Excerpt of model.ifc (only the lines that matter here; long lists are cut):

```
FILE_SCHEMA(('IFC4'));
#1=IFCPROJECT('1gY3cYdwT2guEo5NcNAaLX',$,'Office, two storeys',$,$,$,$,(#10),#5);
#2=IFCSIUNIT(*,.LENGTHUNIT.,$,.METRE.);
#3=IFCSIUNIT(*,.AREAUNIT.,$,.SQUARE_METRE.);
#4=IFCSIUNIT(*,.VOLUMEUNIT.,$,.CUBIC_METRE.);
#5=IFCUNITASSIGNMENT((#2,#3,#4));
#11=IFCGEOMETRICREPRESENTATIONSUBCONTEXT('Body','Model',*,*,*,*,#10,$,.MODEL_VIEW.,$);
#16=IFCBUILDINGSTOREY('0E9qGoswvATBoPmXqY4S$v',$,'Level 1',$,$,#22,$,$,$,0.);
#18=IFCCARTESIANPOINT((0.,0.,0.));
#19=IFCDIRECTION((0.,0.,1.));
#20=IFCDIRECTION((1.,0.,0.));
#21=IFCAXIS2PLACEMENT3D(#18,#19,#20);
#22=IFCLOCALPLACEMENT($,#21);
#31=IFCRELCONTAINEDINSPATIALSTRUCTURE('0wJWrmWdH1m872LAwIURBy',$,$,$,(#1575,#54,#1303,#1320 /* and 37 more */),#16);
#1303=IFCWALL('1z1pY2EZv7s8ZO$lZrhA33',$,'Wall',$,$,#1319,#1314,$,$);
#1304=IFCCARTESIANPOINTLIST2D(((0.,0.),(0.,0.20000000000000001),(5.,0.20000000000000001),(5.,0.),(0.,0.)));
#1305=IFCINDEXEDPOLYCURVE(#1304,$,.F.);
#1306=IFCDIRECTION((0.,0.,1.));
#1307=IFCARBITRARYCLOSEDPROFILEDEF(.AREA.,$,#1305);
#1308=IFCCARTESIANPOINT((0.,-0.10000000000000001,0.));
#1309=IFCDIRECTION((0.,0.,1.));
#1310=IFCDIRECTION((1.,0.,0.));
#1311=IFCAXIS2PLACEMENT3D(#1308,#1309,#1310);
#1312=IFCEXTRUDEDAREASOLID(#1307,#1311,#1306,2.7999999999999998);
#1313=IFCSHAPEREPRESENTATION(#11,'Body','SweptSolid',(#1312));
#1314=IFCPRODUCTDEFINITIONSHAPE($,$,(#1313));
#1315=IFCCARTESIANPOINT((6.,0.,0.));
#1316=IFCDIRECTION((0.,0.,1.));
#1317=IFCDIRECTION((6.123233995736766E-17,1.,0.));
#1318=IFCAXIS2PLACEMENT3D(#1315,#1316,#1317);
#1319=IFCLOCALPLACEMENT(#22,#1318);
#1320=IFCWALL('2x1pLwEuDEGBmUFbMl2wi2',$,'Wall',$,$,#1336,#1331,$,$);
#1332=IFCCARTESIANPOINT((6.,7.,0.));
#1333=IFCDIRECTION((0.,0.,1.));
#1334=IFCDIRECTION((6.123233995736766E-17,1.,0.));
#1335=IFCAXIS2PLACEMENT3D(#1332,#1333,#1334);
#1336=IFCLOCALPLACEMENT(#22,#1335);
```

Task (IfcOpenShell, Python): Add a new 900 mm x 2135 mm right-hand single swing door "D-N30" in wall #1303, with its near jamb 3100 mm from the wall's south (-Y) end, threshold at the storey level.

```python
import numpy as np
import ifcopenshell
import ifcopenshell.api.feature
import ifcopenshell.api.geometry
import ifcopenshell.api.root
import ifcopenshell.api.spatial
import ifcopenshell.geom
import ifcopenshell.util.element
import ifcopenshell.util.placement
import ifcopenshell.util.representation
import ifcopenshell.util.shape
import ifcopenshell.util.unit

model = ifcopenshell.open("model.ifc")
unit_scale = ifcopenshell.util.unit.calculate_unit_scale(model)
settings = ifcopenshell.geom.settings()


def volume(element):
    """Net volume in cubic metres, openings subtracted."""
    shape = ifcopenshell.geom.create_shape(settings, element)
    return ifcopenshell.util.shape.get_volume(shape.geometry)


wall = model.by_guid("1z1pY2EZv7s8ZO$lZrhA33")
storey = ifcopenshell.util.element.get_container(wall, ifc_class="IfcBuildingStorey")
context = ifcopenshell.util.representation.get_context(model, "Model", "Body", "MODEL_VIEW")
before = volume(wall)

width, height, from_end, sill = 0.9, 2.135, 3.1, 0.0  # metres

# The wall runs along its own X axis, and the end named is its -X end.
wall_shape = ifcopenshell.geom.create_shape(settings, wall)
x, y, z = ifcopenshell.util.shape.get_vertices(wall_shape.geometry).T
start = x.min() + from_end
face, thickness = float(y.min()), float(y.max() - y.min())
wall_matrix = ifcopenshell.util.placement.get_local_placement(wall.ObjectPlacement)
level = ifcopenshell.util.placement.get_local_placement(storey.ObjectPlacement)[2, 3]


def in_wall(x, y):
    """Placement at x, y metres in the wall's axes, at sill height."""
    matrix = wall_matrix.copy()
    matrix[:, 3] = wall_matrix @ np.array([x / unit_scale, y / unit_scale, 0.0, 1.0])
    matrix[2, 3] = level + sill / unit_scale
    return matrix


# Opening: a box that overshoots both wall faces by 50 mm.
opening = ifcopenshell.api.root.create_entity(model, ifc_class="IfcOpeningElement", predefined_type="OPENING")
box = ifcopenshell.api.geometry.add_wall_representation(
    model, context=context, length=width, height=height, thickness=thickness + 0.1
)
ifcopenshell.api.geometry.assign_representation(model, product=opening, representation=box)
ifcopenshell.api.geometry.edit_object_placement(model, product=opening, matrix=in_wall(start, face - 0.05), is_si=False)
ifcopenshell.api.feature.add_feature(model, feature=opening, element=wall)

door = ifcopenshell.api.root.create_entity(model, ifc_class="IfcDoor", name="D-N30", predefined_type="DOOR")
door.OverallWidth, door.OverallHeight = width / unit_scale, height / unit_scale
door.OperationType = "SINGLE_SWING_RIGHT"
body = ifcopenshell.api.geometry.add_door_representation(
    model,
    context=context,
    overall_width=door.OverallWidth,
    overall_height=door.OverallHeight,
    operation_type="SINGLE_SWING_RIGHT",
    lining_properties={"LiningDepth": thickness / unit_scale, "ThresholdDepth": thickness / unit_scale},
)
ifcopenshell.api.geometry.assign_representation(model, product=door, representation=body)
ifcopenshell.api.spatial.assign_container(model, products=[door], relating_structure=storey)
ifcopenshell.api.feature.add_filling(model, opening=opening, element=door)

# The lining spans the wall, so the door starts at the wall face.
ifcopenshell.api.geometry.edit_object_placement(model, product=door, matrix=in_wall(start, face), is_si=False)

after = volume(wall)

print(f"wall volume {before:.3f} -> {after:.3f} m3")

model.write("model_updated.ifc")
```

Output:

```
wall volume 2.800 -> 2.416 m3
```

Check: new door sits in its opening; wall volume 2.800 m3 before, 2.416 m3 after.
